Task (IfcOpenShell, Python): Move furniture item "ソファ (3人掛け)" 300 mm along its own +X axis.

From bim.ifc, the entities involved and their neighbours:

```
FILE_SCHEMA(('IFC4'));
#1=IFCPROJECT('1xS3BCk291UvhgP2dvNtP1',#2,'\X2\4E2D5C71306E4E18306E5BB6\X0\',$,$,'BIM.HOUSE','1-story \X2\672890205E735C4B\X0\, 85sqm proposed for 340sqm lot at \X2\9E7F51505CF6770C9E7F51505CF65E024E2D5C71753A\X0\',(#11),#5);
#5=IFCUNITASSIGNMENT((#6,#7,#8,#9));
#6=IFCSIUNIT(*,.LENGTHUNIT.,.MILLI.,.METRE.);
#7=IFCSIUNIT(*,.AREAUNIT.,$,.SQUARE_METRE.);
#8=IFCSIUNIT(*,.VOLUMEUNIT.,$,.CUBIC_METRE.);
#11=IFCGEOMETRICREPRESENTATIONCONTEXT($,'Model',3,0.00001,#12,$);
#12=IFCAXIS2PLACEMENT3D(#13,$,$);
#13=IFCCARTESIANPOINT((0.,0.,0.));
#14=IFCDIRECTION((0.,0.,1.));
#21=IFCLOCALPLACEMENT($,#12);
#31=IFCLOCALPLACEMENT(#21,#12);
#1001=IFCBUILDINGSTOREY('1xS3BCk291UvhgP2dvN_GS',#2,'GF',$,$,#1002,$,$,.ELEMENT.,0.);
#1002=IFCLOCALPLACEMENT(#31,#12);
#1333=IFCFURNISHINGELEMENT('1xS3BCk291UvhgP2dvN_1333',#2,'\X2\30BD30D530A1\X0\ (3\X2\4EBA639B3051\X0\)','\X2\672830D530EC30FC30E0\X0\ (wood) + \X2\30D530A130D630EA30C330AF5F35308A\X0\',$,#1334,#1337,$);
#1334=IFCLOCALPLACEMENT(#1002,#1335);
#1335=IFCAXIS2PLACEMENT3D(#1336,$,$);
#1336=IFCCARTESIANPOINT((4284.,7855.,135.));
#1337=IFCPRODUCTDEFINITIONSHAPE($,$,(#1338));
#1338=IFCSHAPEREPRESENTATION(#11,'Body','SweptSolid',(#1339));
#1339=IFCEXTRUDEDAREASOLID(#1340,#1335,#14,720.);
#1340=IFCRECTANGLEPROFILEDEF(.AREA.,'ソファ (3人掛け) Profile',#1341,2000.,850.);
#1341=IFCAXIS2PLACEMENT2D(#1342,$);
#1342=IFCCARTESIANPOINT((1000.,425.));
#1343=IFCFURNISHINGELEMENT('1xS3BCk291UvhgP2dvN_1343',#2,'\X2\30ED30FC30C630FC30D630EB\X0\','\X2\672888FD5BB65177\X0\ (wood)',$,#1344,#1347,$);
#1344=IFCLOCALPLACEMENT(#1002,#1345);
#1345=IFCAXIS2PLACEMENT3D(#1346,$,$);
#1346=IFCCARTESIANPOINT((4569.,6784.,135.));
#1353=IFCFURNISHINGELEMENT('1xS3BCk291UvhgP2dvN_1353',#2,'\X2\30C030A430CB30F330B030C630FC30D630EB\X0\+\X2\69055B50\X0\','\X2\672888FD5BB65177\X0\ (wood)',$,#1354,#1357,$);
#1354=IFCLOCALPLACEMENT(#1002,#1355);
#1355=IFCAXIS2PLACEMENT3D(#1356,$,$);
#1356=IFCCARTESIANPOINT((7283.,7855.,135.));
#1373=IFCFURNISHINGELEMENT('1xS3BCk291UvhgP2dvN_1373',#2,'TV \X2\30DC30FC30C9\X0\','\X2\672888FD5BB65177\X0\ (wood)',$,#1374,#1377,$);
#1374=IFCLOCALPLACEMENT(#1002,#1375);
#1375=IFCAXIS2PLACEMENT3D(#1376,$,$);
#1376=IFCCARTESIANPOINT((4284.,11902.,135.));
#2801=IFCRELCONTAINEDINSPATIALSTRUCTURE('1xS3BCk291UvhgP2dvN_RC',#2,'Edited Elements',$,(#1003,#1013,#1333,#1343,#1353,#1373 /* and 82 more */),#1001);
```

```python
import ifcopenshell
import ifcopenshell.api.geometry
import ifcopenshell.util.placement
import ifcopenshell.util.unit

model = ifcopenshell.open("bim.ifc")
unit_scale = ifcopenshell.util.unit.calculate_unit_scale(model)

item = model.by_id(1333)
matrix = ifcopenshell.util.placement.get_local_placement(item.ObjectPlacement)
matrix[:3, 3] += matrix[:3, 0] * 0.3 / unit_scale
ifcopenshell.api.geometry.edit_object_placement(model, product=item, matrix=matrix, is_si=False)

print(ifcopenshell.util.placement.get_local_placement(item.ObjectPlacement).round(3) + 0.0)

model.write("bim_edited.ifc")
```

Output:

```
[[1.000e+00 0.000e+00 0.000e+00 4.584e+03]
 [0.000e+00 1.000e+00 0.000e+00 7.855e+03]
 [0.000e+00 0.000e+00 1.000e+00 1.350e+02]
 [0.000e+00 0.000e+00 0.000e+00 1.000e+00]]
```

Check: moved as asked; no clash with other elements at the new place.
